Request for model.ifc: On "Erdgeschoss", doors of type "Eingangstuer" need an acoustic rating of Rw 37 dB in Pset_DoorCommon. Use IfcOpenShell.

First a look at what the model holds.

```python
import ifcopenshell
import ifcopenshell.util.element

model = ifcopenshell.open("model.ifc")
print(model.schema)
storey = next(s for s in model.by_type("IfcBuildingStorey") if s.Name == "Erdgeschoss")
doors = [e for e in ifcopenshell.util.element.get_decomposition(storey) if e.is_a("IfcDoor")]
seen = {}
for e in doors:
    element_type = ifcopenshell.util.element.get_type(e)
    key = (element_type.Name if element_type != e and element_type else None, ifcopenshell.util.element.get_pset(e, "Pset_DoorCommon", "AcousticRating"))
    seen[key] = seen.get(key, 0) + 1
for (name, value), count in sorted(seen.items(), key=str):
    print(count, "x", name, "|", value)
```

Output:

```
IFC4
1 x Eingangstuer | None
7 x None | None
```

```python
import ifcopenshell
import ifcopenshell.api.pset
import ifcopenshell.util.element

model = ifcopenshell.open("model.ifc")

storey = next(s for s in model.by_type("IfcBuildingStorey") if s.Name == "Erdgeschoss")
doors = [e for e in ifcopenshell.util.element.get_decomposition(storey) if e.is_a("IfcDoor")]

count = 0
for e in doors:
    element_type = ifcopenshell.util.element.get_type(e)
    if element_type in (None, e) or element_type.Name != "Eingangstuer":
        continue
    # add_pset returns the element's existing set when there is one.
    pset = ifcopenshell.api.pset.add_pset(model, product=e, name="Pset_DoorCommon")
    ifcopenshell.api.pset.edit_pset(model, pset=pset, properties={"AcousticRating": "Rw 37 dB"})
    count += 1

print(count, "doors updated")

model.write("model_updated.ifc")
```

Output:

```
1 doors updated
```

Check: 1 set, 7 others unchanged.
